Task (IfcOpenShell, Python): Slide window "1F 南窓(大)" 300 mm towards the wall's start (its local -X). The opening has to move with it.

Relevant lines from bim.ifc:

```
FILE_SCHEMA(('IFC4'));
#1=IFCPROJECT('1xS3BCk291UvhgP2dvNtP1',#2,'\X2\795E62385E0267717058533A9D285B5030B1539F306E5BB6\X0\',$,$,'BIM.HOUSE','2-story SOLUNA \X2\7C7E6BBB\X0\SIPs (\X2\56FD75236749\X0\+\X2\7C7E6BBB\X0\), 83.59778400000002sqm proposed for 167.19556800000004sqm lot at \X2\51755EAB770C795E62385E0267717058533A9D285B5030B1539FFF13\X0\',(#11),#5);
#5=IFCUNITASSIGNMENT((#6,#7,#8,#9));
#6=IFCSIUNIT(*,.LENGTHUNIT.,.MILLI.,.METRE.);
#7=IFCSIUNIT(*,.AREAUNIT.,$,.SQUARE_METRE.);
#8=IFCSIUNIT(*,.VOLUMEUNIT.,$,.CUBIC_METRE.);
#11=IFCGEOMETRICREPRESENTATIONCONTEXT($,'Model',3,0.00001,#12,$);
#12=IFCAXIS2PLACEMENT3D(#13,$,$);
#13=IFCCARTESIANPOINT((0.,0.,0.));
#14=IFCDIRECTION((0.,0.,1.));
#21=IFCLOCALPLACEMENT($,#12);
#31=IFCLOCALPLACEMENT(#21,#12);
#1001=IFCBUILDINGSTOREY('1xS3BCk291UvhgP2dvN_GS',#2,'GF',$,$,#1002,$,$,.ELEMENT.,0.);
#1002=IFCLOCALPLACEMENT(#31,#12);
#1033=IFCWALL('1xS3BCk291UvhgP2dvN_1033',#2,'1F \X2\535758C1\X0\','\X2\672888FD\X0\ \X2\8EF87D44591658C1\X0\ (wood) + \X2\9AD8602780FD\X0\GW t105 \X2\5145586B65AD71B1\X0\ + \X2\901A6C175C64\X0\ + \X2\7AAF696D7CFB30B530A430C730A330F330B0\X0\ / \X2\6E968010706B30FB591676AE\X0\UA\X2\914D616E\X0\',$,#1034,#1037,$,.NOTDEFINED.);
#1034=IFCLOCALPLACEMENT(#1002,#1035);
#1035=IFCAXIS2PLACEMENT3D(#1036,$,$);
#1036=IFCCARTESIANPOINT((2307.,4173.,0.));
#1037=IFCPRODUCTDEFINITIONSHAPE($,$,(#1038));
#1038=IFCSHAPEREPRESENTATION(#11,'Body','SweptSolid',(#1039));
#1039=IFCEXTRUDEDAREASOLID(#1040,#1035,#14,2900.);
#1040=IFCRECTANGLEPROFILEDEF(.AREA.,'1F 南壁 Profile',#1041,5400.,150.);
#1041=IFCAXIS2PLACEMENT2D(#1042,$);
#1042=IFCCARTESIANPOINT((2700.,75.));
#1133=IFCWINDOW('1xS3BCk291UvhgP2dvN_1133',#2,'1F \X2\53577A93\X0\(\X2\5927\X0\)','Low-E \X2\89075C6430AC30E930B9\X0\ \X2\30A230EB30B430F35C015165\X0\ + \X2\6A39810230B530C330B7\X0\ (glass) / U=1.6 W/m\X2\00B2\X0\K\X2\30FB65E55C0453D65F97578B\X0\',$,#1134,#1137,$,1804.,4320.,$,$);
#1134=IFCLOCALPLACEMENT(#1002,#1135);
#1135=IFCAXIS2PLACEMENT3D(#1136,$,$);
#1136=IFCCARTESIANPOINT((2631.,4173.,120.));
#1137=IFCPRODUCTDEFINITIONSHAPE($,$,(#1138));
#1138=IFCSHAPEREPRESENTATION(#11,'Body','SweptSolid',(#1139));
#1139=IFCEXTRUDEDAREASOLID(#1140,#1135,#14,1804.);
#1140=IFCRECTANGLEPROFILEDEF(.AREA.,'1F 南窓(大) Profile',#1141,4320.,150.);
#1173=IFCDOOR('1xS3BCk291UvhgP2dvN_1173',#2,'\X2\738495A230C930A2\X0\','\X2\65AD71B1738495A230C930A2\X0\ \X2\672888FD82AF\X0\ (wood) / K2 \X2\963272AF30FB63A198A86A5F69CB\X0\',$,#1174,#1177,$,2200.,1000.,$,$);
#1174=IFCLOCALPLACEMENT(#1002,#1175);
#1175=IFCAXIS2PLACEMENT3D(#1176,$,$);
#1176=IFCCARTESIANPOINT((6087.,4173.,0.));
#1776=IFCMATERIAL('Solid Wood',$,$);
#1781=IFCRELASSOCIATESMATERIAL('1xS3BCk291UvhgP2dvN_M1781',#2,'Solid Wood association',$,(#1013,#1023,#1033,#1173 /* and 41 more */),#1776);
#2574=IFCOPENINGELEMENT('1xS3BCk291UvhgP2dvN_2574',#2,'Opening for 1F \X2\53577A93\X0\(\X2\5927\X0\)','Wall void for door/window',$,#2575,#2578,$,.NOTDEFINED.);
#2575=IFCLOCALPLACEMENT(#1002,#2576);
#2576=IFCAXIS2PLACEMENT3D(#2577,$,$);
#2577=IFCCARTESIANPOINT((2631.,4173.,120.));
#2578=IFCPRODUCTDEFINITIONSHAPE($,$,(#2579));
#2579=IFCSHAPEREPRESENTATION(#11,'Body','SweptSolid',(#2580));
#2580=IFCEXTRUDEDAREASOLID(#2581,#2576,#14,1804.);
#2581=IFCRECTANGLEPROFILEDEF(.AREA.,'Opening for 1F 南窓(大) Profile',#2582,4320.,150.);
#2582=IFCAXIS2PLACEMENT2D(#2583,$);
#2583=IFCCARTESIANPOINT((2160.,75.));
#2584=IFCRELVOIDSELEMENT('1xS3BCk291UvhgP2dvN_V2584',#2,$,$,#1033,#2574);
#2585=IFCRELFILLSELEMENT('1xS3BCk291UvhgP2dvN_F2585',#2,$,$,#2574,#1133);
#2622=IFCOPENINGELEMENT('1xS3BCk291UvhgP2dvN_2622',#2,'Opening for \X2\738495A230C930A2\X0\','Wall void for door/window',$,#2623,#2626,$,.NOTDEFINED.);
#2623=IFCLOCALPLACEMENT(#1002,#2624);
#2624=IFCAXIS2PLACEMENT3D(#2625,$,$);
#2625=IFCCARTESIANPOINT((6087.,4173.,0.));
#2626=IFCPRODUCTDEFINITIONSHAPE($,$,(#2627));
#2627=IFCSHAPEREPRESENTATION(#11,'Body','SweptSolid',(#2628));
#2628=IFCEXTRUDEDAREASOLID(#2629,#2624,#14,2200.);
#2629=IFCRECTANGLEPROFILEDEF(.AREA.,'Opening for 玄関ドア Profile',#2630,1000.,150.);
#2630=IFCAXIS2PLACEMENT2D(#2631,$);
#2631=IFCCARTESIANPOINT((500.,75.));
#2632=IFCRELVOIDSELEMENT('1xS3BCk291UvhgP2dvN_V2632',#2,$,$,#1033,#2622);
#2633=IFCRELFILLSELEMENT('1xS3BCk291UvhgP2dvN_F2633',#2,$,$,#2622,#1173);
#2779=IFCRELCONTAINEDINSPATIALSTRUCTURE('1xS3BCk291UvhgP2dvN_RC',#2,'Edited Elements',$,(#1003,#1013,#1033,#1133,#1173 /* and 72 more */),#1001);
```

```python
import ifcopenshell
import ifcopenshell.api.geometry
import ifcopenshell.util.placement
import ifcopenshell.util.unit

model = ifcopenshell.open("bim.ifc")
unit_scale = ifcopenshell.util.unit.calculate_unit_scale(model)

window = model.by_id(1133)
opening = window.FillsVoids[0].RelatingOpeningElement
wall = opening.VoidsElements[0].RelatingBuildingElement

wall_matrix = ifcopenshell.util.placement.get_local_placement(wall.ObjectPlacement)
shift = wall_matrix[:3, 0] * -0.3 / unit_scale
before = ifcopenshell.util.placement.get_local_placement(window.ObjectPlacement)[:3, 3].copy()

# The window is not placed relative to its opening, so move both.
for product in (opening, window):
    matrix = ifcopenshell.util.placement.get_local_placement(product.ObjectPlacement)
    matrix[:3, 3] += shift
    ifcopenshell.api.geometry.edit_object_placement(model, product=product, matrix=matrix, is_si=False)

after = ifcopenshell.util.placement.get_local_placement(window.ObjectPlacement)[:3, 3]
print("window moved by", (after - before).round(3) + 0.0)

model.write("bim_v2.ifc")
```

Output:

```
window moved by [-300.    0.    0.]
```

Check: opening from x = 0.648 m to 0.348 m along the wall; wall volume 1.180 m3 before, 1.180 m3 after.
